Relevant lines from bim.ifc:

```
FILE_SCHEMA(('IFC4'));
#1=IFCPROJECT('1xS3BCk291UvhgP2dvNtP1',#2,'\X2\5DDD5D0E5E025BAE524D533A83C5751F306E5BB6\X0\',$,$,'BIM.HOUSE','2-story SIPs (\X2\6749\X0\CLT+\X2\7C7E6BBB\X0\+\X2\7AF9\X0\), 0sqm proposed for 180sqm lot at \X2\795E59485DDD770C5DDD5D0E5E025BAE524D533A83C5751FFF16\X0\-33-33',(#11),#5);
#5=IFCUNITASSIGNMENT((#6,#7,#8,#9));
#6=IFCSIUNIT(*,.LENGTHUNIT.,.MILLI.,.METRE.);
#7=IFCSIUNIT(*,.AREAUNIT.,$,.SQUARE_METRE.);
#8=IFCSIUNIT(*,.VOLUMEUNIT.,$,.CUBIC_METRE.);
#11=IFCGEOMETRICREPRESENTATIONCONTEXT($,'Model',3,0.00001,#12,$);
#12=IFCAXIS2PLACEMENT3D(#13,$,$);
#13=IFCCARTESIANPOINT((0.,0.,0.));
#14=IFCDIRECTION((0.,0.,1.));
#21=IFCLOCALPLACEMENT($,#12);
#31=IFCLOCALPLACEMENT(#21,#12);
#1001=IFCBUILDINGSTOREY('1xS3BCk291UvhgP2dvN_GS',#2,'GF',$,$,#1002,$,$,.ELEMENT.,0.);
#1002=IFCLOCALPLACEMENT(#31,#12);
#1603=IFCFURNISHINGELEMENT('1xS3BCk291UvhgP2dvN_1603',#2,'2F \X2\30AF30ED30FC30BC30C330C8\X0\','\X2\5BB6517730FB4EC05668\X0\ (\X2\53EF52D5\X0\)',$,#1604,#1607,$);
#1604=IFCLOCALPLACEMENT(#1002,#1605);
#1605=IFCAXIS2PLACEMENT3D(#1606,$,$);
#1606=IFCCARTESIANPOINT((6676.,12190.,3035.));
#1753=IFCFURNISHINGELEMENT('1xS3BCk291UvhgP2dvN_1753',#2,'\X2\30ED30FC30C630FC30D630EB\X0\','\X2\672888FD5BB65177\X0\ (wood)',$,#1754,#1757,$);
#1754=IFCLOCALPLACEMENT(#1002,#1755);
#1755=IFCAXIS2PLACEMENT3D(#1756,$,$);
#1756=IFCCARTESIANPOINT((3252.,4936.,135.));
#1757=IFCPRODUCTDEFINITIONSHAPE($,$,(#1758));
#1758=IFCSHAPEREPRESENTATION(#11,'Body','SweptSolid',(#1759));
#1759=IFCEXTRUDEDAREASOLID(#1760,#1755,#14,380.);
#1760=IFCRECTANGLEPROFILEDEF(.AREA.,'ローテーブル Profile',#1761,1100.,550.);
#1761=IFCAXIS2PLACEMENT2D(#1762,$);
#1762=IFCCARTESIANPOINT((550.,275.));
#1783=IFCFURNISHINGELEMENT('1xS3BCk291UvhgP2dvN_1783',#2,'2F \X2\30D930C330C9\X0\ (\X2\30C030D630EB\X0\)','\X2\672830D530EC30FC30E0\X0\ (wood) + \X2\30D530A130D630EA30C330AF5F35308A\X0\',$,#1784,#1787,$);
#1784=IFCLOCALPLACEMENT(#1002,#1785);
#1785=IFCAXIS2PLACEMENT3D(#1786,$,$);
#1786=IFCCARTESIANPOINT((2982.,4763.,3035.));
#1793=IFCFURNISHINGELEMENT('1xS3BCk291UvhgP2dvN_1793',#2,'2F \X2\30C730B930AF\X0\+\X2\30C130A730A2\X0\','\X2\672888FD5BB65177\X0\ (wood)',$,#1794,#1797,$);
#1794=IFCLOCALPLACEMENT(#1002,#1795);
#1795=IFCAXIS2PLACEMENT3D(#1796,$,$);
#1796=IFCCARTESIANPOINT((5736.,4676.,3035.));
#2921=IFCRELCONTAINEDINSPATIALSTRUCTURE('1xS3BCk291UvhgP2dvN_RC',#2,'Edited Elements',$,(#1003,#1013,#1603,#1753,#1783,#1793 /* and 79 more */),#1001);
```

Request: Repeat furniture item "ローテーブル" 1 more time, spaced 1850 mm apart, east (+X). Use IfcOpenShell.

```python
import numpy as np
import ifcopenshell
import ifcopenshell.api.geometry
import ifcopenshell.api.root
import ifcopenshell.util.element
import ifcopenshell.util.placement

model = ifcopenshell.open("bim.ifc")


def reuse_history(source, copy):
    """copy_class also copies each property set's owner history, people and application; keep the originals."""
    for rel in copy.IsDefinedBy:
        if rel.is_a("IfcRelDefinesByProperties") and (history := rel.RelatingPropertyDefinition.OwnerHistory):
            rel.RelatingPropertyDefinition.OwnerHistory = source.OwnerHistory
            ifcopenshell.util.element.remove_deep2(model, history)


source = model.by_guid("1xS3BCk291UvhgP2dvN_1753")
base = ifcopenshell.util.placement.get_local_placement(source.ObjectPlacement)
step = np.array([1.0, 0.0, 0.0]) * 1850.0

for i in range(1, 2):
    copy = ifcopenshell.api.root.copy_class(model, product=source)
    copy.Representation = ifcopenshell.util.element.copy_deep(
        model, source.Representation, exclude=["IfcGeometricRepresentationContext", "IfcRepresentationMap"]
    )
    reuse_history(source, copy)
    matrix = base.copy()
    matrix[:3, 3] += i * step
    print("added at", matrix[:3, 3].round(3) + 0.0)
    ifcopenshell.api.geometry.edit_object_placement(model, product=copy, matrix=matrix, is_si=False)

model.write("bim_updated.ifc")
```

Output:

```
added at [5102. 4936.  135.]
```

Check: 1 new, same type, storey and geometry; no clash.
